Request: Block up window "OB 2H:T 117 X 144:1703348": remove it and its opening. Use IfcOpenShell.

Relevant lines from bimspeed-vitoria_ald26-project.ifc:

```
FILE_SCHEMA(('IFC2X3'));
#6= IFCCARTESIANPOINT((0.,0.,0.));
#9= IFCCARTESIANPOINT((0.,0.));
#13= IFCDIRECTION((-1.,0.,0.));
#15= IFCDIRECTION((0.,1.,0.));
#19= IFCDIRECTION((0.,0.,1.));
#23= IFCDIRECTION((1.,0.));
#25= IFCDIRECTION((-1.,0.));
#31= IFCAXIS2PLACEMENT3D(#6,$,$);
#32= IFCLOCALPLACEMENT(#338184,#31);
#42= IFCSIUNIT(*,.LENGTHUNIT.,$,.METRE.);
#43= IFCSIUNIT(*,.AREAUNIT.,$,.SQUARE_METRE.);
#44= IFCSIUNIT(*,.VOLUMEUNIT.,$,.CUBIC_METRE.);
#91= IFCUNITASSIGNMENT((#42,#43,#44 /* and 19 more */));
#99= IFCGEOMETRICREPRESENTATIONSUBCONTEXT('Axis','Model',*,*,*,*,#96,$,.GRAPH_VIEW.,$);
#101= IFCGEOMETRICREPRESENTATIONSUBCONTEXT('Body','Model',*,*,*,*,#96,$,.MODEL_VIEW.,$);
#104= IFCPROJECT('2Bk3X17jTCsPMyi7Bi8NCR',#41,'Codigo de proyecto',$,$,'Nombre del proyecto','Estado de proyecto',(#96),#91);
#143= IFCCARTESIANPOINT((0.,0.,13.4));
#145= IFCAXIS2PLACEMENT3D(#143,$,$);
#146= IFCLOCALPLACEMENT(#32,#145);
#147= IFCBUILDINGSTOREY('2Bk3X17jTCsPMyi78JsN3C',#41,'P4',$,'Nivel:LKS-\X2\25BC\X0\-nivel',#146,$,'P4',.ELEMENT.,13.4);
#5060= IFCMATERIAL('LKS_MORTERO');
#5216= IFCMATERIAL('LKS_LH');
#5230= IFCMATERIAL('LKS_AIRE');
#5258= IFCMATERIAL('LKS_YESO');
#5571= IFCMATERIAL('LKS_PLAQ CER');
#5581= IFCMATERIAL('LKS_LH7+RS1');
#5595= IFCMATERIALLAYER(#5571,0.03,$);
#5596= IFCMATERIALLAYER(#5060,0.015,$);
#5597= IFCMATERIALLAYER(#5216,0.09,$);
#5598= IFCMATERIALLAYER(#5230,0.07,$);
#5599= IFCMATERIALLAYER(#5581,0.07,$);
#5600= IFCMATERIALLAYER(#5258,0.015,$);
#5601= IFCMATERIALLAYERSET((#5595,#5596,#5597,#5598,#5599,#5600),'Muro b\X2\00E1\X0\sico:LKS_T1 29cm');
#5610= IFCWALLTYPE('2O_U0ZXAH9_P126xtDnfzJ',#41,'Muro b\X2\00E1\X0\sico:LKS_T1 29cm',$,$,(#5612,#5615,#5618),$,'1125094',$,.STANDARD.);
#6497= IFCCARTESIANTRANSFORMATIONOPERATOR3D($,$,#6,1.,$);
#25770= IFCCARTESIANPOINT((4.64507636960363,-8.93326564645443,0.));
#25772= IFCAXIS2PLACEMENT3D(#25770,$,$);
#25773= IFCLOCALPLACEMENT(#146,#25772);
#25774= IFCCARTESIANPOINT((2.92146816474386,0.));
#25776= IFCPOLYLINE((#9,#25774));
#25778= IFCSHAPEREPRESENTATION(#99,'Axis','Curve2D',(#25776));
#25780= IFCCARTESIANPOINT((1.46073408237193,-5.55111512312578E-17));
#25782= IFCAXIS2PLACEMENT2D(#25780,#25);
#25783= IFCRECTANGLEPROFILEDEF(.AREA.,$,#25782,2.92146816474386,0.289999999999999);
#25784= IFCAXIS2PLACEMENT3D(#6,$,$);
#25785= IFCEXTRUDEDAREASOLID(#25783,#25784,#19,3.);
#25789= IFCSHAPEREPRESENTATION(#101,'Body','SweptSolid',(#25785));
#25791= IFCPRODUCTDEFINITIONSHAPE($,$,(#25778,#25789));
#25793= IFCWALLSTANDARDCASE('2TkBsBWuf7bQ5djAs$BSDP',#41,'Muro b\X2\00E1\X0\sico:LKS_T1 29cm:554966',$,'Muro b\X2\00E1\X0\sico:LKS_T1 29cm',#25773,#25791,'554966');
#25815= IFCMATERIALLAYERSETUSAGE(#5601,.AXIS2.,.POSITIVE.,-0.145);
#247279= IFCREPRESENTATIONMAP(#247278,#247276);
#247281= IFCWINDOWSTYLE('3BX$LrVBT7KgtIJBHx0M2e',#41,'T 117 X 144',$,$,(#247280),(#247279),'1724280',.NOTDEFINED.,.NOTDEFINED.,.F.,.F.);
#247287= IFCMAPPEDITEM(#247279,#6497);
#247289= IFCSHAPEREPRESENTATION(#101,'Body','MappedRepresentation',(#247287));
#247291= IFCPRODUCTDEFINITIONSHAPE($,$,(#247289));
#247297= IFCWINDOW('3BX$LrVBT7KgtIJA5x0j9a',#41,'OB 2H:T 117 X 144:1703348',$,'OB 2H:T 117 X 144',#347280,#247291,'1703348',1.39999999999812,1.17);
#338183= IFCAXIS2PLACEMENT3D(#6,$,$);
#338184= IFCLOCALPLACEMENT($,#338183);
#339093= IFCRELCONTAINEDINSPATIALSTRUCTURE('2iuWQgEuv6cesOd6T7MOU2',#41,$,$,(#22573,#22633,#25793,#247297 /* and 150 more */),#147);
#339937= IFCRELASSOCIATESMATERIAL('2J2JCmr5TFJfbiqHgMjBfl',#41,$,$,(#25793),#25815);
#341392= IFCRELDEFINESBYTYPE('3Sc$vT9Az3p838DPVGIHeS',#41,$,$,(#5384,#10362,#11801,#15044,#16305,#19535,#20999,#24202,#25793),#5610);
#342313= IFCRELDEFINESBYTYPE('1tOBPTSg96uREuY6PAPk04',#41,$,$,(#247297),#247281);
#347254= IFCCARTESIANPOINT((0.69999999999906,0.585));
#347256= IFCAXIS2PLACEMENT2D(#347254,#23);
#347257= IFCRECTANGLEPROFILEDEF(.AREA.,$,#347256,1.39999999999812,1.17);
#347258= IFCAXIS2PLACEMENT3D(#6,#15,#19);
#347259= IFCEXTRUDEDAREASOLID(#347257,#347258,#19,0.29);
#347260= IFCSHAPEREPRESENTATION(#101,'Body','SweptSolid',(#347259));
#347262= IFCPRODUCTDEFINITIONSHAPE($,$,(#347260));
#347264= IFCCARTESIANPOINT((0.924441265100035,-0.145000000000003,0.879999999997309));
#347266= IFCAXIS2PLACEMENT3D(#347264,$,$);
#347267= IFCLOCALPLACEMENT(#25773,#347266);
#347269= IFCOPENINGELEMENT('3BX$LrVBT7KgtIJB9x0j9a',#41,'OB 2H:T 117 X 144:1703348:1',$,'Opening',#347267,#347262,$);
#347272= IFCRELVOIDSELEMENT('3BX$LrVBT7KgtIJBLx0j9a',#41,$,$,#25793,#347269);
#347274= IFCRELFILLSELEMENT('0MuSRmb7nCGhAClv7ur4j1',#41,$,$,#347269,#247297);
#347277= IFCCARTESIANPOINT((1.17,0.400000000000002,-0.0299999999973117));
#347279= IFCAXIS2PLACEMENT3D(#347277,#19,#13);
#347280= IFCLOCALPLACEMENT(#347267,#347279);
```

```python
import ifcopenshell
import ifcopenshell.api.feature
import ifcopenshell.api.root
import ifcopenshell.geom
import ifcopenshell.util.shape

model = ifcopenshell.open("bimspeed-vitoria_ald26-project.ifc")
settings = ifcopenshell.geom.settings()


def volume(element):
    """Net volume in cubic metres, openings subtracted."""
    shape = ifcopenshell.geom.create_shape(settings, element)
    return ifcopenshell.util.shape.get_volume(shape.geometry)


window = model.by_guid("3BX$LrVBT7KgtIJA5x0j9a")
opening = window.FillsVoids[0].RelatingOpeningElement
wall = opening.VoidsElements[0].RelatingBuildingElement
before = volume(wall)

ifcopenshell.api.root.remove_product(model, product=window)
ifcopenshell.api.feature.remove_feature(model, feature=opening)

after = volume(wall)

print(f"wall volume {before:.3f} -> {after:.3f} m3")

model.write("bimspeed-vitoria_ald26-project-out.ifc")
```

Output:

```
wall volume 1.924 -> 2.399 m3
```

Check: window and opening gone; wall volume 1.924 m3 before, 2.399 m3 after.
